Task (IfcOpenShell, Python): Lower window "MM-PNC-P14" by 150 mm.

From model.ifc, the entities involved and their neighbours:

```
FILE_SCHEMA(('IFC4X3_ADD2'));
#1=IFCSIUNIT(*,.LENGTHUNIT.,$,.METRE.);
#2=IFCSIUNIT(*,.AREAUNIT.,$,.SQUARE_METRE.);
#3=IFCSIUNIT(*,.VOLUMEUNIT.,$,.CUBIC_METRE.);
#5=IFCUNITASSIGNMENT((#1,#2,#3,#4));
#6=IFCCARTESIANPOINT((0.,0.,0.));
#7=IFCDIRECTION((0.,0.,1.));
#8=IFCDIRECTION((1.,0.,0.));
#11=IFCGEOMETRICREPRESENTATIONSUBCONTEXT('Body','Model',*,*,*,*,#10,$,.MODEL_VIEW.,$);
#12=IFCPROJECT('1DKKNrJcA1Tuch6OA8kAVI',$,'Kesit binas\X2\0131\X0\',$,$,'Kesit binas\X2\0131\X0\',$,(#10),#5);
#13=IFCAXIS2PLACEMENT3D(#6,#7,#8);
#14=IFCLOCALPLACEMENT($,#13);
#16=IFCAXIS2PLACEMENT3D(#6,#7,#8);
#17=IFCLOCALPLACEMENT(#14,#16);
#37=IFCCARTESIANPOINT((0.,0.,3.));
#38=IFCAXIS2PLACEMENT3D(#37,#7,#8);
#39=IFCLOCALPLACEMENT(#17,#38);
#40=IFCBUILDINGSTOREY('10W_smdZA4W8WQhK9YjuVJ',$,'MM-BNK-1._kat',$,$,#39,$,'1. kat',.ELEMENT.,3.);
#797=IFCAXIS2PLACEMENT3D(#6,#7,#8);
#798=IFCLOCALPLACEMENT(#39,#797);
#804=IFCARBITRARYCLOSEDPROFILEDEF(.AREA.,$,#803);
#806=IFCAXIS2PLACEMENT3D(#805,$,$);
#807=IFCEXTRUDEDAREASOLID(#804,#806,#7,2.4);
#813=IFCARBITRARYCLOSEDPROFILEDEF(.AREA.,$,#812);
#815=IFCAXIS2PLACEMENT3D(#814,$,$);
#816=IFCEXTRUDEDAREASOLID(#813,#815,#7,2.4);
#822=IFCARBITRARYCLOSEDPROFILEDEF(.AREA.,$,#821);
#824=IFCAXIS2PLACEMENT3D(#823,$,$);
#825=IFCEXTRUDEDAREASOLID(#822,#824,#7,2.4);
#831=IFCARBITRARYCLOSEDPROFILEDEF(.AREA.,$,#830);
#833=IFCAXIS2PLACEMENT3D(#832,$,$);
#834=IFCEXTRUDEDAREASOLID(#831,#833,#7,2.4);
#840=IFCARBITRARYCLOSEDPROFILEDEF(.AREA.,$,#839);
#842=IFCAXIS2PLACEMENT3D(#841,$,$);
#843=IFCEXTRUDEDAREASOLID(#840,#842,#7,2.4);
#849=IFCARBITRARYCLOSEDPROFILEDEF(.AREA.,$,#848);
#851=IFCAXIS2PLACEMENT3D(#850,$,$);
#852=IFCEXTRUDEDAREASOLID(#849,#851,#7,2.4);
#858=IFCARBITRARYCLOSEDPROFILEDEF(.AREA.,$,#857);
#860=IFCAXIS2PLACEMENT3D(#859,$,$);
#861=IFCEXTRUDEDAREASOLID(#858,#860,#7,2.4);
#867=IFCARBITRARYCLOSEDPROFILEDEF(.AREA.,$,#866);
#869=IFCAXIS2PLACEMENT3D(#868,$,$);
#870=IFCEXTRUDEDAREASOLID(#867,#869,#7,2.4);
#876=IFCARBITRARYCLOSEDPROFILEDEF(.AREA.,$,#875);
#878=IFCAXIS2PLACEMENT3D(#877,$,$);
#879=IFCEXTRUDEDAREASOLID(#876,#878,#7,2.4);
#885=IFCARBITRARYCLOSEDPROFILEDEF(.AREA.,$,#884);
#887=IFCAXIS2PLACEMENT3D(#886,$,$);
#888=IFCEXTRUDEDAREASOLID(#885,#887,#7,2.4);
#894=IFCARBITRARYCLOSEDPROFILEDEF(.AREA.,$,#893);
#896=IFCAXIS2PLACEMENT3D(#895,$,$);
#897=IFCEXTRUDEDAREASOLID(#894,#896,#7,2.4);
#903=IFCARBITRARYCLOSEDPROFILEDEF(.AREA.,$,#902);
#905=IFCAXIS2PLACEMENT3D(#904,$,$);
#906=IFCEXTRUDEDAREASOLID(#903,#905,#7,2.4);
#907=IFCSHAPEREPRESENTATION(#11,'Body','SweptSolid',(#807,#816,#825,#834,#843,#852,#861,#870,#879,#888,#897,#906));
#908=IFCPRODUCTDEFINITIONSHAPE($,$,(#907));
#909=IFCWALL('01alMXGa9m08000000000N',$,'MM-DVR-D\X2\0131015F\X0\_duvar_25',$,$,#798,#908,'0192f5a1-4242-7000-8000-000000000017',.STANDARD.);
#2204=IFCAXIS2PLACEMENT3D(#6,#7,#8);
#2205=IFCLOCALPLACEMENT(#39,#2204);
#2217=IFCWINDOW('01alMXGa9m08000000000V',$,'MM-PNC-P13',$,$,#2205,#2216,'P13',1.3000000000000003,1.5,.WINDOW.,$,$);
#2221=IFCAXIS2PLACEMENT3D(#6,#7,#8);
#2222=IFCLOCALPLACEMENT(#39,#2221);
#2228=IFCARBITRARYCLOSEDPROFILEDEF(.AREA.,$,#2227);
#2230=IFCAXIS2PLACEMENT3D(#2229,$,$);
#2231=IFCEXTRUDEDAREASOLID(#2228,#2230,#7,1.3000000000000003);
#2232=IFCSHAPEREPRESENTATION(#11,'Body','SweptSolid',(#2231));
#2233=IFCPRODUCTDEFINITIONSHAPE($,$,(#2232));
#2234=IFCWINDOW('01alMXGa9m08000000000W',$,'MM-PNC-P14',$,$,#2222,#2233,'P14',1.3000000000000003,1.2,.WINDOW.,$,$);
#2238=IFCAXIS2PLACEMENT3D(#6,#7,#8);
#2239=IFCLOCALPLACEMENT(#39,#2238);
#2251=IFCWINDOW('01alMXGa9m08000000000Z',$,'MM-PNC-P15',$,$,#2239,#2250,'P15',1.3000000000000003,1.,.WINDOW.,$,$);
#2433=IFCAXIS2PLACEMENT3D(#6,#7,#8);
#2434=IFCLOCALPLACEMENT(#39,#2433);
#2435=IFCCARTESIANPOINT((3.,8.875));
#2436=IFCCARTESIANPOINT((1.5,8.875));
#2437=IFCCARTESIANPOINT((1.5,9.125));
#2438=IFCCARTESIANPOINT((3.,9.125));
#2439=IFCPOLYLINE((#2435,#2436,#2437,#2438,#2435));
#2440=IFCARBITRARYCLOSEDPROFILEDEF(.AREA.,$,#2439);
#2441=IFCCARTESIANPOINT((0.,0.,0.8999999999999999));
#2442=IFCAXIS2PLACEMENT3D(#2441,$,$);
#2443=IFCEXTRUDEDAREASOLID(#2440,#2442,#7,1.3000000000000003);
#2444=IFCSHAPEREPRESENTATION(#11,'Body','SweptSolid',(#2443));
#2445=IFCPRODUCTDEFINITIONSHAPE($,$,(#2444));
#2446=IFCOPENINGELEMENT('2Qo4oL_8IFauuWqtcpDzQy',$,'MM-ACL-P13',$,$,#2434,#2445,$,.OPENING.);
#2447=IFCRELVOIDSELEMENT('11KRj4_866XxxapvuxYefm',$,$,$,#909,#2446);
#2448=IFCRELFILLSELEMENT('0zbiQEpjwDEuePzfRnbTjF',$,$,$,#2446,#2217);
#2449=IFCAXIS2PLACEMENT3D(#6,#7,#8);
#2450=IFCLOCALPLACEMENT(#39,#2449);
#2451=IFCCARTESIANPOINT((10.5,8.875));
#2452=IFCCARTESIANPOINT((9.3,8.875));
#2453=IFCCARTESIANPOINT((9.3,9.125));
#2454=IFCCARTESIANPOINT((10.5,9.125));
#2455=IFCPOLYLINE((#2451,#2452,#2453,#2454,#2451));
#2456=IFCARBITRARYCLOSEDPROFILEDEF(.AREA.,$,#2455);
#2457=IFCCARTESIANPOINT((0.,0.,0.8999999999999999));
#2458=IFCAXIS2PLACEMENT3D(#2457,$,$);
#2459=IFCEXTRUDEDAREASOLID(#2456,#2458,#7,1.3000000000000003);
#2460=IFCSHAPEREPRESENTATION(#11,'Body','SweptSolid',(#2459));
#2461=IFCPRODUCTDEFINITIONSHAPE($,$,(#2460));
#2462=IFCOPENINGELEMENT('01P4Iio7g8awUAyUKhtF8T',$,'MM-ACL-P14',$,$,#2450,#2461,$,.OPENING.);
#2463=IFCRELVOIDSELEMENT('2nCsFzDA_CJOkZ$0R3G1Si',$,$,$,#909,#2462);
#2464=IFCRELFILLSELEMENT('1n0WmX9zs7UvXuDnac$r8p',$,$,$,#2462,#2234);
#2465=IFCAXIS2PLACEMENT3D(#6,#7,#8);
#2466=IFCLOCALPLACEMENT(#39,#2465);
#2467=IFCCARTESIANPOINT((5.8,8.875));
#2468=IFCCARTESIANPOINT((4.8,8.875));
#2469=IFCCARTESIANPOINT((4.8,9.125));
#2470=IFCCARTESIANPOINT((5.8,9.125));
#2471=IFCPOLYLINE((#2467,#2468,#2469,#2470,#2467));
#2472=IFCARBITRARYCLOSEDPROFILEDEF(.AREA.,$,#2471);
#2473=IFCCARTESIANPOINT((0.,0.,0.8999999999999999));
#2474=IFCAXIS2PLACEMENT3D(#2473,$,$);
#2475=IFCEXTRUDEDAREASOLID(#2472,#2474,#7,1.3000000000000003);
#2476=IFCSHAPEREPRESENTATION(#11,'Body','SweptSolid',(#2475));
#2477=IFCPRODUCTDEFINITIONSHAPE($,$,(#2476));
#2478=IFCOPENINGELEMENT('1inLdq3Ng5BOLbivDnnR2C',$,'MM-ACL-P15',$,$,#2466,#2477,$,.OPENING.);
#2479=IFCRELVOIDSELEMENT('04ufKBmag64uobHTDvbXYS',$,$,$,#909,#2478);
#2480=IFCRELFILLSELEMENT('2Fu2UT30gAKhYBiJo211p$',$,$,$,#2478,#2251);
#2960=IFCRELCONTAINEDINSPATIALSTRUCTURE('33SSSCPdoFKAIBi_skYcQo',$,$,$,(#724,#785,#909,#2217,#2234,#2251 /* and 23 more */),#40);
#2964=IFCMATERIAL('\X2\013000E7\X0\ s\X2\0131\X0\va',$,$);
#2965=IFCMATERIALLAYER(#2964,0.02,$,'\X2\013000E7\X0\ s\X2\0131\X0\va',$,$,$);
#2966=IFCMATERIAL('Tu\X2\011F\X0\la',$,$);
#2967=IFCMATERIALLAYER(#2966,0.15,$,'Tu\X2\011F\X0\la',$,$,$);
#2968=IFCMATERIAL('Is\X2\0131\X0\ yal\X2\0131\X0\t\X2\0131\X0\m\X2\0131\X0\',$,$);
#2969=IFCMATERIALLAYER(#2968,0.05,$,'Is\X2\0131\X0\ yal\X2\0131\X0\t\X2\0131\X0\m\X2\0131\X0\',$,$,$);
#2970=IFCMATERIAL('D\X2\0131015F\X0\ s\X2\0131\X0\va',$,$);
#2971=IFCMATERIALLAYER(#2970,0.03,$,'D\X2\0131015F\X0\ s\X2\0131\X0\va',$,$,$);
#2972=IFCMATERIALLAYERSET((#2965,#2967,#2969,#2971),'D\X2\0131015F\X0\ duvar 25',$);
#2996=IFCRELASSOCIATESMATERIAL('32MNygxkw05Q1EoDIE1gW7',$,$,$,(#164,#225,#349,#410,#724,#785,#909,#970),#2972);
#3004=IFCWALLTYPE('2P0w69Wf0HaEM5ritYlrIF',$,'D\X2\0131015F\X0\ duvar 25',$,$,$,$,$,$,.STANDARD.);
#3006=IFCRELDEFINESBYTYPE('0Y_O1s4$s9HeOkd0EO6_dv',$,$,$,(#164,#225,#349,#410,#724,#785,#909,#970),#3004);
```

```python
import numpy as np
import ifcopenshell
import ifcopenshell.api.geometry
import ifcopenshell.util.placement
import ifcopenshell.util.unit

model = ifcopenshell.open("model.ifc")
unit_scale = ifcopenshell.util.unit.calculate_unit_scale(model)

window = model.by_guid("01alMXGa9m08000000000W")
opening = window.FillsVoids[0].RelatingOpeningElement
dz = -0.15 / unit_scale

shift = np.array([0.0, 0.0, dz])
# The window is not placed relative to its opening, so move both.
for product in (opening, window):
    matrix = ifcopenshell.util.placement.get_local_placement(product.ObjectPlacement)
    matrix[:3, 3] += shift
    ifcopenshell.api.geometry.edit_object_placement(model, product=product, matrix=matrix, is_si=False)

print(f"moved by {dz * unit_scale:+.3f} m")

model.write("model_v2.ifc")
```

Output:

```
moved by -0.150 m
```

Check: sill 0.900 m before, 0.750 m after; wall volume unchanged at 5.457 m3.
